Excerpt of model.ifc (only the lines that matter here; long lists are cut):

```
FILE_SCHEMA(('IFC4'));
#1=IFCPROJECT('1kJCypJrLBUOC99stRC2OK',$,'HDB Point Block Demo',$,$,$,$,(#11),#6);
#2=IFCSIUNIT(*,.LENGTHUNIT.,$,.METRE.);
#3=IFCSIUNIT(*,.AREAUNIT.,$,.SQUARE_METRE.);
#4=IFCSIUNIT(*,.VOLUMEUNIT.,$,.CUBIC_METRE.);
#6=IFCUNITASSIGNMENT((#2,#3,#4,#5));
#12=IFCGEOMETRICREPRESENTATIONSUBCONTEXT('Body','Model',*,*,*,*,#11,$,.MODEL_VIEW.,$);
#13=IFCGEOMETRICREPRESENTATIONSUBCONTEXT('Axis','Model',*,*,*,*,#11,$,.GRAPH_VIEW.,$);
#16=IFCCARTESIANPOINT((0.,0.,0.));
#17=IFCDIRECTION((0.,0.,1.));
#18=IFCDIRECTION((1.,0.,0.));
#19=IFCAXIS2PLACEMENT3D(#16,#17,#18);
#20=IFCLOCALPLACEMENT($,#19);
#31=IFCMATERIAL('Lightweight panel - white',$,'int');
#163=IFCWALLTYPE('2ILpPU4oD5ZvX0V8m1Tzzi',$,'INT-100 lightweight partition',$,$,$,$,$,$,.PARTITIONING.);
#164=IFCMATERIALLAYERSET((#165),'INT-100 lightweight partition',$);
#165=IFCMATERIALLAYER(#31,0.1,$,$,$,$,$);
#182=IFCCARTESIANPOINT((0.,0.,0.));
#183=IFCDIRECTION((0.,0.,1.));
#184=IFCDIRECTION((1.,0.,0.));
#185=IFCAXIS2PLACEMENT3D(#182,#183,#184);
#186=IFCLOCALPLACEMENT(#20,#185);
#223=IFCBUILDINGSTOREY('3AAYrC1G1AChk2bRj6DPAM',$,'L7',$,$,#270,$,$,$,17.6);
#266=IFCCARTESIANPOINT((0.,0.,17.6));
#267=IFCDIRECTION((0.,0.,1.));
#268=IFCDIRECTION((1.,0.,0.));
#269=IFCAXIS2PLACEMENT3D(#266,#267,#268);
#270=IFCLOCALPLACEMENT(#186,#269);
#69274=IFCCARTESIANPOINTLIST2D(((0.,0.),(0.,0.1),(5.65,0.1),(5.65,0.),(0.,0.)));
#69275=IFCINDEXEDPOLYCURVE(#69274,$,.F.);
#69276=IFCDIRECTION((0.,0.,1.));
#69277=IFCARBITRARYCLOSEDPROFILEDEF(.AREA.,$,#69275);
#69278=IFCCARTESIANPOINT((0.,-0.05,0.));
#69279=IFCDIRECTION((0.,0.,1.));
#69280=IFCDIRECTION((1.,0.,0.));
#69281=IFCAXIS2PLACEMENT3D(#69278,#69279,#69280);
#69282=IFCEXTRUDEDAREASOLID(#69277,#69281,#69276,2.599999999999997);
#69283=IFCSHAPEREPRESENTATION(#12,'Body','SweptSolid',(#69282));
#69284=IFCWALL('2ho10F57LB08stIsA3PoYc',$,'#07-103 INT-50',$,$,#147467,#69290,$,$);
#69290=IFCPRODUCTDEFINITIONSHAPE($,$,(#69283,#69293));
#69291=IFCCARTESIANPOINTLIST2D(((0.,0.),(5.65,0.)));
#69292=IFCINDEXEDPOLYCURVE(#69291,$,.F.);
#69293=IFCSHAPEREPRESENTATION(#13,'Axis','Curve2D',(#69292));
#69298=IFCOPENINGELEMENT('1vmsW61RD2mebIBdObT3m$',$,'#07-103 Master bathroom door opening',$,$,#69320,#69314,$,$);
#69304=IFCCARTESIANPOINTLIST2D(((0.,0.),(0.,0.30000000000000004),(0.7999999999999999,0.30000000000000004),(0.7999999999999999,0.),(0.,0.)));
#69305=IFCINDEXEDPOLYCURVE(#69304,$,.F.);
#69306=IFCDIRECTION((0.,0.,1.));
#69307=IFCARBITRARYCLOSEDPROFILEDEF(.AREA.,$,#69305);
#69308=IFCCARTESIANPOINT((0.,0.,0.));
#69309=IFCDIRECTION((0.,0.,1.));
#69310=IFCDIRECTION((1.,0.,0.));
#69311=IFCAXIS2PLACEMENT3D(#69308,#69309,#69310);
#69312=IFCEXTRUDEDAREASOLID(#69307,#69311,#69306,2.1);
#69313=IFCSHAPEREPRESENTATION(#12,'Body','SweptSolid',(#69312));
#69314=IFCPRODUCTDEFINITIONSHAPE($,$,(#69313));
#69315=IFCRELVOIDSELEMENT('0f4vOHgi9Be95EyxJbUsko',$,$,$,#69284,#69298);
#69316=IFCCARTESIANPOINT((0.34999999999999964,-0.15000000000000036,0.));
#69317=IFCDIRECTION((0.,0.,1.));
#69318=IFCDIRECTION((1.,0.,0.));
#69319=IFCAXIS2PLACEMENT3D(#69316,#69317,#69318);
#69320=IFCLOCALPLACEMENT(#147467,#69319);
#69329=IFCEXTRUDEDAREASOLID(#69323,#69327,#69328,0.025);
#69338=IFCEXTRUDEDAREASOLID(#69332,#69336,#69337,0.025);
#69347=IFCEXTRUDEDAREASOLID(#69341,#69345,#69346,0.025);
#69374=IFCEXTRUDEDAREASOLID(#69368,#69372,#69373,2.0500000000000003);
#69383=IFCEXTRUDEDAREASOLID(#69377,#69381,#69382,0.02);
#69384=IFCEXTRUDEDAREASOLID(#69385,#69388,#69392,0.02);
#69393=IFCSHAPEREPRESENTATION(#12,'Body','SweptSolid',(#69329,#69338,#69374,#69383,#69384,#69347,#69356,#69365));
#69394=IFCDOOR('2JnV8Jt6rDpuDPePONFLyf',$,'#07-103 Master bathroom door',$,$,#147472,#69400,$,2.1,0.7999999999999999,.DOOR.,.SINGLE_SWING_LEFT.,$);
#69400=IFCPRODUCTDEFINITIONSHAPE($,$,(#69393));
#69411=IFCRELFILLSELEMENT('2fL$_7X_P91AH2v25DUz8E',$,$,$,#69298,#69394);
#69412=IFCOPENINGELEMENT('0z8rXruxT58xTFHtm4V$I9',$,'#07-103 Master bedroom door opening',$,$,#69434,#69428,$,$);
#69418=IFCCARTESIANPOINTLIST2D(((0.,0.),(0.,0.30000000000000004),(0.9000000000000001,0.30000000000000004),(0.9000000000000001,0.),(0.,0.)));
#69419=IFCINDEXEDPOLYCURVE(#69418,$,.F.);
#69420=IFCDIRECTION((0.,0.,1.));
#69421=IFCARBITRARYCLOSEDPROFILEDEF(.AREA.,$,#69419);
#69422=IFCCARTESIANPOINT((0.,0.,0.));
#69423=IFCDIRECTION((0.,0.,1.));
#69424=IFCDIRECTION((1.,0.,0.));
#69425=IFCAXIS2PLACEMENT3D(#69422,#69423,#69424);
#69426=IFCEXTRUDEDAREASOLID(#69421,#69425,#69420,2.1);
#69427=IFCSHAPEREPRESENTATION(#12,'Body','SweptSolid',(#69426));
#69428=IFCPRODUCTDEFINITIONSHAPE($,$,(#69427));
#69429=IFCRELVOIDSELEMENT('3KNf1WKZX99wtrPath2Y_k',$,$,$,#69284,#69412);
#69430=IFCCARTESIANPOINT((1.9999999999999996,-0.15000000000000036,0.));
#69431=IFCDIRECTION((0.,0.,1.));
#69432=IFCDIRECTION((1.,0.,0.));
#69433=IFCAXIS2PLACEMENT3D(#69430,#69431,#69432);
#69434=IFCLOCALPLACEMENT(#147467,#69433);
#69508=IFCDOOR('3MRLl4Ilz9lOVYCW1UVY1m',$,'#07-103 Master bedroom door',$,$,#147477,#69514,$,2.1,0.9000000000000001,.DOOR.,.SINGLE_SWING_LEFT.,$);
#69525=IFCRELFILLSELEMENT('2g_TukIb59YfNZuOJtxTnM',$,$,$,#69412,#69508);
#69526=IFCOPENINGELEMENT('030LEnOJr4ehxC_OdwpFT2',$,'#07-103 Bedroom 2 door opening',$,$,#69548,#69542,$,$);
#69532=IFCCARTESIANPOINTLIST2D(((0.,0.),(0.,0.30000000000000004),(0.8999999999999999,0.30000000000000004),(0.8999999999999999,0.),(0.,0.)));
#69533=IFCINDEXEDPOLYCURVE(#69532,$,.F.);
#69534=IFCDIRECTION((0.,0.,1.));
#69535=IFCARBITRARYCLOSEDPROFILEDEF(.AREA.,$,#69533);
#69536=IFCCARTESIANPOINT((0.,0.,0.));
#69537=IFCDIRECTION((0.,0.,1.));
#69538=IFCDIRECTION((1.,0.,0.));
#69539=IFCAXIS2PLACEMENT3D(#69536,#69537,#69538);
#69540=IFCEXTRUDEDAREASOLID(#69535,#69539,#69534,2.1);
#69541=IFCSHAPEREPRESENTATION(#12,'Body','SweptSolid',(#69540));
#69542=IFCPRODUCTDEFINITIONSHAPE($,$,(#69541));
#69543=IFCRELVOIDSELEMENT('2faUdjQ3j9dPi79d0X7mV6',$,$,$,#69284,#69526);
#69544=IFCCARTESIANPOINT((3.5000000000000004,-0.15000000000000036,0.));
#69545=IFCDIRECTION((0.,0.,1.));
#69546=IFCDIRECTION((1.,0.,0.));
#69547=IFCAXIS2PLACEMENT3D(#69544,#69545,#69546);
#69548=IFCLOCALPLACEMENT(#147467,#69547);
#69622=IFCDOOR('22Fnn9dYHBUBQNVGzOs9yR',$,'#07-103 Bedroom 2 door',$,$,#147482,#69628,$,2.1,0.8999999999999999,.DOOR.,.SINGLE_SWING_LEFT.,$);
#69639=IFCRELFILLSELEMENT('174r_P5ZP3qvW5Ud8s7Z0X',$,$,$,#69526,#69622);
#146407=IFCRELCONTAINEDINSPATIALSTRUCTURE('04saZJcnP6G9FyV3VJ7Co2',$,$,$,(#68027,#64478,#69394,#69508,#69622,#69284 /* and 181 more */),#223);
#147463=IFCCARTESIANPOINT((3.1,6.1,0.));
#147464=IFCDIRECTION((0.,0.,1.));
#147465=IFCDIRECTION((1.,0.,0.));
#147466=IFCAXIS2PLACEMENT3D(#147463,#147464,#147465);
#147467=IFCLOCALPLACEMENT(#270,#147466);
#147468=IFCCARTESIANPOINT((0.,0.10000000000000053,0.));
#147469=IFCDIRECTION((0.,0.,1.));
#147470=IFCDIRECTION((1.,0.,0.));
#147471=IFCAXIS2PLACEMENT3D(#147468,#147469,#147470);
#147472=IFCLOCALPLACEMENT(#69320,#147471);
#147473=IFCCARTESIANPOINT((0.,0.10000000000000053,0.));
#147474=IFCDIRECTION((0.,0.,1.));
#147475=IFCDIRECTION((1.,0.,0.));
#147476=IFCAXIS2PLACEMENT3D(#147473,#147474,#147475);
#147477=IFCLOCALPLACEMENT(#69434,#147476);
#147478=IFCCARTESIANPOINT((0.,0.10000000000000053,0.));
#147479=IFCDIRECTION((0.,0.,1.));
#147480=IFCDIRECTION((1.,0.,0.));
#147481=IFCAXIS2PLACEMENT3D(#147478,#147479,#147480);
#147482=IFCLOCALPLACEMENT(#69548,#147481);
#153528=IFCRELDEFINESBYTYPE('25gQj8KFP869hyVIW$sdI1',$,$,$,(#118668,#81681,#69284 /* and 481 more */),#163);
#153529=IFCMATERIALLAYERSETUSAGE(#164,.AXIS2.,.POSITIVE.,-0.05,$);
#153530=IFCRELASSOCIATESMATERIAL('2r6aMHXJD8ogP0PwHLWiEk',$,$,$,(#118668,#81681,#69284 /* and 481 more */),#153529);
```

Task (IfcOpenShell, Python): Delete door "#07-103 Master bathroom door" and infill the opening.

```python
import ifcopenshell
import ifcopenshell.api.feature
import ifcopenshell.api.root
import ifcopenshell.geom
import ifcopenshell.util.shape

model = ifcopenshell.open("model.ifc")
settings = ifcopenshell.geom.settings()


def volume(element):
    """Net volume in cubic metres, openings subtracted."""
    shape = ifcopenshell.geom.create_shape(settings, element)
    return ifcopenshell.util.shape.get_volume(shape.geometry)


door = model.by_id(69394)
opening = door.FillsVoids[0].RelatingOpeningElement
wall = opening.VoidsElements[0].RelatingBuildingElement
before = volume(wall)

ifcopenshell.api.root.remove_product(model, product=door)
ifcopenshell.api.feature.remove_feature(model, feature=opening)

after = volume(wall)

print(f"wall volume {before:.3f} -> {after:.3f} m3")

model.write("model_edited.ifc")
```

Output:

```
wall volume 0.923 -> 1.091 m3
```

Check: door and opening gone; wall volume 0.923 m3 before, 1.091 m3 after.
